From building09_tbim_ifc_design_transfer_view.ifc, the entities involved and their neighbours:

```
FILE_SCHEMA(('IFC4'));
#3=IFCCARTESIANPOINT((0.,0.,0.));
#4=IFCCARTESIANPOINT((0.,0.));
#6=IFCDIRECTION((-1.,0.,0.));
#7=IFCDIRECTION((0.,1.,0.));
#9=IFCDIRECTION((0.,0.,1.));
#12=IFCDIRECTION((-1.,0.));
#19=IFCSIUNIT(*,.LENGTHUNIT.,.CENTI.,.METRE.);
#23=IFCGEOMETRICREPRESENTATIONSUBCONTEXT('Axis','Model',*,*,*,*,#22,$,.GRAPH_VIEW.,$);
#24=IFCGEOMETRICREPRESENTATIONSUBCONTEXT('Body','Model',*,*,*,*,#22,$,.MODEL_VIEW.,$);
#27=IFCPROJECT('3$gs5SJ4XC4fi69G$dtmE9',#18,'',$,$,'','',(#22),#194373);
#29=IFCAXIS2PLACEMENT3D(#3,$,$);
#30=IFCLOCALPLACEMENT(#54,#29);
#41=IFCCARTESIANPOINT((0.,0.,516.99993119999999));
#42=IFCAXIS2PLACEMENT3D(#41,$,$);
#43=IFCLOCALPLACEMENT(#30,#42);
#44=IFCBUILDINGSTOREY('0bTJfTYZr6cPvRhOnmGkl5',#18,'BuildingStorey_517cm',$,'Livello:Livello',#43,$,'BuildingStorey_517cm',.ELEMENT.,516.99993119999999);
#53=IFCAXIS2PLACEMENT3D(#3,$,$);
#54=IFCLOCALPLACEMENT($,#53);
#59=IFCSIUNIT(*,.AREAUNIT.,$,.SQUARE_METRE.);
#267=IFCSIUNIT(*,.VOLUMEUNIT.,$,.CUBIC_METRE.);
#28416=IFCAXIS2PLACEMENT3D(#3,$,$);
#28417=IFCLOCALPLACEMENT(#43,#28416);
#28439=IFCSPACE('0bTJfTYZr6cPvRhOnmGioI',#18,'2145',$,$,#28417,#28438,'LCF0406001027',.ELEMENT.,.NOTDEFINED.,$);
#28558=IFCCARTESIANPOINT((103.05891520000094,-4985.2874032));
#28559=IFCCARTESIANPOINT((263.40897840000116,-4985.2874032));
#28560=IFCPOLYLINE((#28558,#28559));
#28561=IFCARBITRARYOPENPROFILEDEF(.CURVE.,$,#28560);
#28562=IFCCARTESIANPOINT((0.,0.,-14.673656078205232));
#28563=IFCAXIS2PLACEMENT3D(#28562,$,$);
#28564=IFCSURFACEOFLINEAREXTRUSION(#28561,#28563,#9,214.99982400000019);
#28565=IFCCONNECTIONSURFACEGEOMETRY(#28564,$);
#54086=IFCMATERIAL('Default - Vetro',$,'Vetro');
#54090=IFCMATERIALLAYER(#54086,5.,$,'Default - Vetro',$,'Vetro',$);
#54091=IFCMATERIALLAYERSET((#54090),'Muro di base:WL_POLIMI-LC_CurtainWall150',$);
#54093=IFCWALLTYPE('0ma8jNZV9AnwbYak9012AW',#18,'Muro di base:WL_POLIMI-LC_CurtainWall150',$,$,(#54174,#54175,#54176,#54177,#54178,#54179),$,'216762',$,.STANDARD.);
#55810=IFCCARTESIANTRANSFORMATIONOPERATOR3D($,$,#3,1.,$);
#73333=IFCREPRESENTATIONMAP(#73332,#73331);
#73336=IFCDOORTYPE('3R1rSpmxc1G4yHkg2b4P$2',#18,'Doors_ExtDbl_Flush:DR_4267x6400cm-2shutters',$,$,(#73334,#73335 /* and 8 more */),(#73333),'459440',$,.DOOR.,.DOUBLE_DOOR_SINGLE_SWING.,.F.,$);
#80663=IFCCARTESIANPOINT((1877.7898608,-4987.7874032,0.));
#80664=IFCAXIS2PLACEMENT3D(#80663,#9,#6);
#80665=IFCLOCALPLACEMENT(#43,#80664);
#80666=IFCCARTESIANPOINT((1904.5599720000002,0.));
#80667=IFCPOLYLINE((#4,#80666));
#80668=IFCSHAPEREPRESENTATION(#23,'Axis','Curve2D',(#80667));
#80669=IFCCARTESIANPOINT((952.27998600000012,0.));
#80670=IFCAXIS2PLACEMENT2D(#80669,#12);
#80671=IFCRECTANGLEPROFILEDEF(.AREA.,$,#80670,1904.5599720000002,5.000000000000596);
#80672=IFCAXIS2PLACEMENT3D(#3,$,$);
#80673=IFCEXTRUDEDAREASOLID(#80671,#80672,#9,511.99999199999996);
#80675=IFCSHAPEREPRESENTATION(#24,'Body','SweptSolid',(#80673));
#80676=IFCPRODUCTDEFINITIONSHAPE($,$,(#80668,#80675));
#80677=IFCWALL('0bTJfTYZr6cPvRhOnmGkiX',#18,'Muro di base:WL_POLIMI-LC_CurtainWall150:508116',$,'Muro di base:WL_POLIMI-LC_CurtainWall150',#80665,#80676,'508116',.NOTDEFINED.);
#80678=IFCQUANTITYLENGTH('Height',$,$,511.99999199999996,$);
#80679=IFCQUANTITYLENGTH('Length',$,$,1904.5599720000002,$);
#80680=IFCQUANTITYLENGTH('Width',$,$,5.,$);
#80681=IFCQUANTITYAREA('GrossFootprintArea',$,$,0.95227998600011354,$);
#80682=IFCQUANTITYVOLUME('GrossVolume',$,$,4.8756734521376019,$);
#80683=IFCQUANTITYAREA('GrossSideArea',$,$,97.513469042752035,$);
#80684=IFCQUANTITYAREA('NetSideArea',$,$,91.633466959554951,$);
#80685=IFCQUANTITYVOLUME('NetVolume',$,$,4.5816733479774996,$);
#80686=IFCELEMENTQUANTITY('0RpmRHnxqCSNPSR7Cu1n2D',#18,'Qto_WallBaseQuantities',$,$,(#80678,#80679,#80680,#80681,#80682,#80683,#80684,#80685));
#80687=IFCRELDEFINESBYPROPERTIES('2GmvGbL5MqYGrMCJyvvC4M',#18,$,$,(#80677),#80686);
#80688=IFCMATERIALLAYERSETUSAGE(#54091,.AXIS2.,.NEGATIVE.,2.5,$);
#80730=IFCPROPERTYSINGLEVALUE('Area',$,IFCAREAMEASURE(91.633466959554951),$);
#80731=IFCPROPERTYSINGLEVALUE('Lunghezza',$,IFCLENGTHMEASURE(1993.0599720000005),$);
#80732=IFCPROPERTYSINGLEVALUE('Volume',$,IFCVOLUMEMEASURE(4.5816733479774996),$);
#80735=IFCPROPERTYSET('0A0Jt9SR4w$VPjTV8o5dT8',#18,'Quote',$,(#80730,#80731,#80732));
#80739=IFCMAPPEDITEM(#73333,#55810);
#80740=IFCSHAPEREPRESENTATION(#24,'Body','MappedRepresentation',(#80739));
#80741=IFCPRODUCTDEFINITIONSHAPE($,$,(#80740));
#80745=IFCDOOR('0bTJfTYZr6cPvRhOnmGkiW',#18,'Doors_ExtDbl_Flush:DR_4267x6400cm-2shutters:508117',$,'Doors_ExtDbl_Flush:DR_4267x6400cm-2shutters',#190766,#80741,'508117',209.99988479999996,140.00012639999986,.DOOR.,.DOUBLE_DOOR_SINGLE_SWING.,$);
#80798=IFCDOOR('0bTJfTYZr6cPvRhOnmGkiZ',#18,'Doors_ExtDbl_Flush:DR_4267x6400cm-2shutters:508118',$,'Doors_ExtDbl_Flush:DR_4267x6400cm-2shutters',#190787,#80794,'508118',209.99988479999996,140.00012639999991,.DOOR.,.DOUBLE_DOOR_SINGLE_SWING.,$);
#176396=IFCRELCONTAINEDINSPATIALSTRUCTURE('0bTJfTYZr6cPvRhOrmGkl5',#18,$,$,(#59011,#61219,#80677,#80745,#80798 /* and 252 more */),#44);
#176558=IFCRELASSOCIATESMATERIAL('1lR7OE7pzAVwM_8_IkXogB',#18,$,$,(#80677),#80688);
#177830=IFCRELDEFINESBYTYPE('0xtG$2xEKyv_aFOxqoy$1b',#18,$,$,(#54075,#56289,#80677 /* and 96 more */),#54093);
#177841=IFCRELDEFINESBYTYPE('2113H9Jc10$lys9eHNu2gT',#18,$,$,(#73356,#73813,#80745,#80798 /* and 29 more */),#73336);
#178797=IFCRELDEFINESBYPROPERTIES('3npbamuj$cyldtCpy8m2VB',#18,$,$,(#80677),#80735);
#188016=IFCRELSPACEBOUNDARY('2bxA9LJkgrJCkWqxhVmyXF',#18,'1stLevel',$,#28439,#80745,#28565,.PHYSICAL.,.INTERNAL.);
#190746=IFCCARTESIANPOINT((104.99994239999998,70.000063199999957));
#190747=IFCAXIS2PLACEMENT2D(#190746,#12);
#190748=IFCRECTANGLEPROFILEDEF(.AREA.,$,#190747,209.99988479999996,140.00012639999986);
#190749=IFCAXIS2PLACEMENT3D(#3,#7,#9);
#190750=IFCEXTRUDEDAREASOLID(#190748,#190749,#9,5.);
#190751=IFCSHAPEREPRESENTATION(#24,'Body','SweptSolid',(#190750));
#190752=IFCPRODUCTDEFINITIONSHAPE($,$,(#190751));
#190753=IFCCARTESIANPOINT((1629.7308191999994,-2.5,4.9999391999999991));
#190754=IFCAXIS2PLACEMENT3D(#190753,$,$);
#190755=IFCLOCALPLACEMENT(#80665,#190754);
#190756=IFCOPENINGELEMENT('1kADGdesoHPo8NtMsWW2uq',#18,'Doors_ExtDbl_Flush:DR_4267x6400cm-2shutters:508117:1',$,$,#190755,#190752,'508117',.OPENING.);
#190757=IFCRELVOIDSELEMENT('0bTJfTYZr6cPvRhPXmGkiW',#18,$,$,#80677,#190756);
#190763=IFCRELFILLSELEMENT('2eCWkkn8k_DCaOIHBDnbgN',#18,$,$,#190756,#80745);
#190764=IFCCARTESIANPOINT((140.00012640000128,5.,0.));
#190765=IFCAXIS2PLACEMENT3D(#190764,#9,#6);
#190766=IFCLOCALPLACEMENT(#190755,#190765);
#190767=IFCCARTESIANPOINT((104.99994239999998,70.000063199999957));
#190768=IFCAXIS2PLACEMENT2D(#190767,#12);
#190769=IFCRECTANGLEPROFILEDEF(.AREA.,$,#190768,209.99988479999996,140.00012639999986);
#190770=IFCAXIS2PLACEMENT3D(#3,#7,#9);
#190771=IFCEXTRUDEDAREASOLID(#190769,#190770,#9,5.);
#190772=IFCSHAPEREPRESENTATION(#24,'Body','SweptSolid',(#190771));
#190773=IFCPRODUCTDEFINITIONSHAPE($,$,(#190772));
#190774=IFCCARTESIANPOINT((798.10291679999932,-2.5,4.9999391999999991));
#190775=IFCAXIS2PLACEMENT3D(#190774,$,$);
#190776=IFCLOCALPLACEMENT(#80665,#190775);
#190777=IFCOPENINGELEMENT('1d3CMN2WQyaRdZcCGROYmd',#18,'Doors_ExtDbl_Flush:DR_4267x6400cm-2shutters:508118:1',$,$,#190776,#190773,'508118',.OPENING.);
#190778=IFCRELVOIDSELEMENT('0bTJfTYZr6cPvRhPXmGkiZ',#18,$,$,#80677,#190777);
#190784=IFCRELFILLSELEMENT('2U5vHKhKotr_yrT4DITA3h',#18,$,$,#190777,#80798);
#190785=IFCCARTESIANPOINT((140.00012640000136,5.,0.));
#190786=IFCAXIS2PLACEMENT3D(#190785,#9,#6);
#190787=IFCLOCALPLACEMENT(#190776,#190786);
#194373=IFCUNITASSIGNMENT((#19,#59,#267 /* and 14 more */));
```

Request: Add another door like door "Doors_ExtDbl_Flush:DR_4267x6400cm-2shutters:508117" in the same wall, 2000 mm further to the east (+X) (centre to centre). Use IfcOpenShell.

```python
import numpy as np
import ifcopenshell
import ifcopenshell.api.feature
import ifcopenshell.api.geometry
import ifcopenshell.api.pset
import ifcopenshell.api.root
import ifcopenshell.geom
import ifcopenshell.util.element
import ifcopenshell.util.placement
import ifcopenshell.util.shape
import ifcopenshell.util.unit

model = ifcopenshell.open("building09_tbim_ifc_design_transfer_view.ifc")
unit_scale = ifcopenshell.util.unit.calculate_unit_scale(model)
area_scale = ifcopenshell.util.unit.calculate_unit_scale(model, "AREAUNIT")
volume_scale = ifcopenshell.util.unit.calculate_unit_scale(model, "VOLUMEUNIT")
settings = ifcopenshell.geom.settings()


def volume(element):
    """Net volume in cubic metres, openings subtracted."""
    shape = ifcopenshell.geom.create_shape(settings, element)
    return ifcopenshell.util.shape.get_volume(shape.geometry)


def reuse_history(source, copy):
    """copy_class also copies each property set's owner history, people and application; keep the originals."""
    for rel in copy.IsDefinedBy:
        if rel.is_a("IfcRelDefinesByProperties") and (history := rel.RelatingPropertyDefinition.OwnerHistory):
            rel.RelatingPropertyDefinition.OwnerHistory = source.OwnerHistory
            ifcopenshell.util.element.remove_deep2(model, history)


door = model.by_guid("0bTJfTYZr6cPvRhOnmGkiW")
opening = door.FillsVoids[0].RelatingOpeningElement
wall = opening.VoidsElements[0].RelatingBuildingElement
before = volume(wall)
shift = ifcopenshell.util.placement.get_local_placement(wall.ObjectPlacement)[:3, 0] * -2 / unit_scale

# copy_class copies the void relationship, type, container and properties, but no geometry.
new_opening = ifcopenshell.api.root.copy_class(model, product=opening)
new_opening.Representation = ifcopenshell.util.element.copy_deep(
    model, opening.Representation, exclude=["IfcGeometricRepresentationContext", "IfcRepresentationMap"]
)
new_opening.Name = "Doors_ExtDbl_Flush:DR_4267x6400cm-2shutters"
new_opening.Tag = None
reuse_history(opening, new_opening)
new_door = ifcopenshell.api.root.copy_class(model, product=door)
new_door.Representation = ifcopenshell.util.element.copy_deep(
    model, door.Representation, exclude=["IfcGeometricRepresentationContext", "IfcRepresentationMap"]
)
new_door.Name = "Doors_ExtDbl_Flush:DR_4267x6400cm-2shutters"
new_door.Tag = None
reuse_history(door, new_door)
ifcopenshell.api.feature.add_filling(model, opening=new_opening, element=new_door)

for old, new in ((opening, new_opening), (door, new_door)):
    matrix = ifcopenshell.util.placement.get_local_placement(old.ObjectPlacement)
    matrix[:3, 3] += shift
    ifcopenshell.api.geometry.edit_object_placement(model, product=new, matrix=matrix, is_si=False)

# The copied space boundaries still share their surfaces with the original.
for rel in new_door.ProvidesBoundaries:
    if rel.ConnectionGeometry:
        rel.ConnectionGeometry = ifcopenshell.util.element.copy_deep(model, rel.ConnectionGeometry)

# Space boundary surfaces are stored in each space's coordinates; move them too.
for rel in new_door.ProvidesBoundaries:
    if not rel.ConnectionGeometry:
        continue
    surface = rel.ConnectionGeometry.SurfaceOnRelatingElement
    space_matrix = ifcopenshell.util.placement.get_local_placement(rel.RelatingSpace.ObjectPlacement)
    point = np.array(surface.Position.Location.Coordinates) + space_matrix[:3, :3].T @ shift
    surface.Position = model.createIfcAxis2Placement3D(
        model.createIfcCartesianPoint(point.tolist()), surface.Position.Axis, surface.Position.RefDirection
    )

after = volume(wall)
thickness = 0.05  # wall thickness in metres

# Update the wall's stored quantities.
qto = model.by_id(ifcopenshell.util.element.get_pset(wall, "Qto_WallBaseQuantities", should_inherit=False)["id"])
ifcopenshell.api.pset.edit_qto(model, qto=qto, properties={
    "NetSideArea": after / thickness / area_scale,
    "NetVolume": after / volume_scale,
})
pset = model.by_id(ifcopenshell.util.element.get_pset(wall, "Quote", should_inherit=False)["id"])
ifcopenshell.api.pset.edit_pset(model, pset=pset, properties={
    "Area": model.create_entity("IfcAreaMeasure", after / thickness / area_scale),
    "Volume": model.create_entity("IfcVolumeMeasure", after / volume_scale),
})

print(f"wall volume {before:.3f} -> {after:.3f} m3")

model.write("building09_tbim_ifc_design_transfer_view_rev.ifc")
```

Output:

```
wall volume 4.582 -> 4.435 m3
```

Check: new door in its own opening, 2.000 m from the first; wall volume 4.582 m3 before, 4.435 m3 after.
